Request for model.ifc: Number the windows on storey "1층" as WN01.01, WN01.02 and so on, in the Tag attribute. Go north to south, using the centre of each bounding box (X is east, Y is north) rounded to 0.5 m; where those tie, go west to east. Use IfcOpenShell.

First a look at what the model holds.

```python
import ifcopenshell
import ifcopenshell.util.element
import ifcopenshell.util.placement

model = ifcopenshell.open("model.ifc")
print(model.schema)
storey = next(s for s in model.by_type("IfcBuildingStorey") if s.Name == "1층")
windows = [e for e in ifcopenshell.util.element.get_decomposition(storey) if e.is_a("IfcWindow")]
for e in sorted(windows, key=lambda e: e.id()):
    origin = ifcopenshell.util.placement.get_local_placement(e.ObjectPlacement)[:3, 3]
    print(e.id(), e.Tag, e.Name, origin.round(2) + 0.0, sep=" | ")
```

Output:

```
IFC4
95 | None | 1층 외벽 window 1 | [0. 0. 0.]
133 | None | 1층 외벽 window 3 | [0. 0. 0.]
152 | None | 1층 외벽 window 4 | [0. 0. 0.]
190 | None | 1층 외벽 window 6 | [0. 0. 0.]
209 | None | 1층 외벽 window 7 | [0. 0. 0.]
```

```python
import ifcopenshell
import ifcopenshell.geom
import ifcopenshell.util.element
import ifcopenshell.util.shape

model = ifcopenshell.open("model.ifc")
settings = ifcopenshell.geom.settings()
settings.set("use-world-coords", True)


def centre(element):
    shape = ifcopenshell.geom.create_shape(settings, element)
    return ifcopenshell.util.shape.get_bbox_centroid(shape.geometry)


storey = next(s for s in model.by_type("IfcBuildingStorey") if s.Name == "1층")
windows = [e for e in ifcopenshell.util.element.get_decomposition(storey) if e.is_a("IfcWindow")]

# Insertion points can sit at a corner or the storey origin, so sort by the geometry (in metres).
centres = {e: centre(e) for e in windows}
windows.sort(key=lambda e: (-round(centres[e][1] / 0.5), centres[e][0]))

for i, e in enumerate(windows, start=1):
    number = f"WN01.{i:02d}"
    e.Tag = number
    print(e.id(), number)

model.write("model_rev.ifc")
```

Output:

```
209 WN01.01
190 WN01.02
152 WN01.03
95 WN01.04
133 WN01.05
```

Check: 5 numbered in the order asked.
